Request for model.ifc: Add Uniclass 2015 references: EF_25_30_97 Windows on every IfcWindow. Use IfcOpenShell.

First a look at what the model holds.

```python
import ifcopenshell

model = ifcopenshell.open("model.ifc")
print(model.schema)
print("classifications:", [c.Name for c in model.by_type("IfcClassification")])
for ifc_class in ("IfcDoor", "IfcRoof", "IfcStair", "IfcWall", "IfcWindow"):
    print(ifc_class, len(model.by_type(ifc_class)))
```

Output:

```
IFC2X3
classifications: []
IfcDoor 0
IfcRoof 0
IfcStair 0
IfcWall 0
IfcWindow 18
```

```python
import ifcopenshell
import ifcopenshell.api.classification

model = ifcopenshell.open("model.ifc")

# IFC2X3 requires Source and Edition and has no link from the project to the system.
system = model.create_entity("IfcClassification", Source="NBS", Edition="2015", Name="Uniclass 2015")

codes = {
    "IfcWindow": ("EF_25_30_97", "Windows"),
}
for ifc_class, (code, name) in codes.items():
    products = model.by_type(ifc_class)
    ifcopenshell.api.classification.add_reference(
        model, products=products, classification=system, identification=code, name=name
    )
    print(code, len(products))

model.write("model_edited.ifc")
```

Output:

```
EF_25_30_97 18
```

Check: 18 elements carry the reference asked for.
